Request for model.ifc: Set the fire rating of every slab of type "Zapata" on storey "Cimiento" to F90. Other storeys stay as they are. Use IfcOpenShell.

First a look at what the model holds.

```python
import ifcopenshell
import ifcopenshell.util.element

model = ifcopenshell.open("model.ifc")
print(model.schema)
storey = next(s for s in model.by_type("IfcBuildingStorey") if s.Name == "Cimiento")
slabs = [e for e in ifcopenshell.util.element.get_decomposition(storey) if e.is_a("IfcSlab")]
seen = {}
for e in slabs:
    element_type = ifcopenshell.util.element.get_type(e)
    key = (element_type.Name if element_type != e and element_type else None, ifcopenshell.util.element.get_pset(e, "Pset_SlabCommon", "FireRating"))
    seen[key] = seen.get(key, 0) + 1
for (name, value), count in sorted(seen.items(), key=str):
    print(count, "x", name, "|", value)
```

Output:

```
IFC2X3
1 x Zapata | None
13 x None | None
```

```python
import ifcopenshell
import ifcopenshell.api.pset
import ifcopenshell.util.element

model = ifcopenshell.open("model.ifc")

storey = next(s for s in model.by_type("IfcBuildingStorey") if s.Name == "Cimiento")
slabs = [e for e in ifcopenshell.util.element.get_decomposition(storey) if e.is_a("IfcSlab")]

count = 0
for e in slabs:
    element_type = ifcopenshell.util.element.get_type(e)
    if element_type in (None, e) or element_type.Name != "Zapata":
        continue
    # add_pset returns the element's existing set when there is one.
    pset = ifcopenshell.api.pset.add_pset(model, product=e, name="Pset_SlabCommon")
    ifcopenshell.api.pset.edit_pset(model, pset=pset, properties={"FireRating": "F90"})
    count += 1

print(count, "slabs updated")

model.write("model-out.ifc")
```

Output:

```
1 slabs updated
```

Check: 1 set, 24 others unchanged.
